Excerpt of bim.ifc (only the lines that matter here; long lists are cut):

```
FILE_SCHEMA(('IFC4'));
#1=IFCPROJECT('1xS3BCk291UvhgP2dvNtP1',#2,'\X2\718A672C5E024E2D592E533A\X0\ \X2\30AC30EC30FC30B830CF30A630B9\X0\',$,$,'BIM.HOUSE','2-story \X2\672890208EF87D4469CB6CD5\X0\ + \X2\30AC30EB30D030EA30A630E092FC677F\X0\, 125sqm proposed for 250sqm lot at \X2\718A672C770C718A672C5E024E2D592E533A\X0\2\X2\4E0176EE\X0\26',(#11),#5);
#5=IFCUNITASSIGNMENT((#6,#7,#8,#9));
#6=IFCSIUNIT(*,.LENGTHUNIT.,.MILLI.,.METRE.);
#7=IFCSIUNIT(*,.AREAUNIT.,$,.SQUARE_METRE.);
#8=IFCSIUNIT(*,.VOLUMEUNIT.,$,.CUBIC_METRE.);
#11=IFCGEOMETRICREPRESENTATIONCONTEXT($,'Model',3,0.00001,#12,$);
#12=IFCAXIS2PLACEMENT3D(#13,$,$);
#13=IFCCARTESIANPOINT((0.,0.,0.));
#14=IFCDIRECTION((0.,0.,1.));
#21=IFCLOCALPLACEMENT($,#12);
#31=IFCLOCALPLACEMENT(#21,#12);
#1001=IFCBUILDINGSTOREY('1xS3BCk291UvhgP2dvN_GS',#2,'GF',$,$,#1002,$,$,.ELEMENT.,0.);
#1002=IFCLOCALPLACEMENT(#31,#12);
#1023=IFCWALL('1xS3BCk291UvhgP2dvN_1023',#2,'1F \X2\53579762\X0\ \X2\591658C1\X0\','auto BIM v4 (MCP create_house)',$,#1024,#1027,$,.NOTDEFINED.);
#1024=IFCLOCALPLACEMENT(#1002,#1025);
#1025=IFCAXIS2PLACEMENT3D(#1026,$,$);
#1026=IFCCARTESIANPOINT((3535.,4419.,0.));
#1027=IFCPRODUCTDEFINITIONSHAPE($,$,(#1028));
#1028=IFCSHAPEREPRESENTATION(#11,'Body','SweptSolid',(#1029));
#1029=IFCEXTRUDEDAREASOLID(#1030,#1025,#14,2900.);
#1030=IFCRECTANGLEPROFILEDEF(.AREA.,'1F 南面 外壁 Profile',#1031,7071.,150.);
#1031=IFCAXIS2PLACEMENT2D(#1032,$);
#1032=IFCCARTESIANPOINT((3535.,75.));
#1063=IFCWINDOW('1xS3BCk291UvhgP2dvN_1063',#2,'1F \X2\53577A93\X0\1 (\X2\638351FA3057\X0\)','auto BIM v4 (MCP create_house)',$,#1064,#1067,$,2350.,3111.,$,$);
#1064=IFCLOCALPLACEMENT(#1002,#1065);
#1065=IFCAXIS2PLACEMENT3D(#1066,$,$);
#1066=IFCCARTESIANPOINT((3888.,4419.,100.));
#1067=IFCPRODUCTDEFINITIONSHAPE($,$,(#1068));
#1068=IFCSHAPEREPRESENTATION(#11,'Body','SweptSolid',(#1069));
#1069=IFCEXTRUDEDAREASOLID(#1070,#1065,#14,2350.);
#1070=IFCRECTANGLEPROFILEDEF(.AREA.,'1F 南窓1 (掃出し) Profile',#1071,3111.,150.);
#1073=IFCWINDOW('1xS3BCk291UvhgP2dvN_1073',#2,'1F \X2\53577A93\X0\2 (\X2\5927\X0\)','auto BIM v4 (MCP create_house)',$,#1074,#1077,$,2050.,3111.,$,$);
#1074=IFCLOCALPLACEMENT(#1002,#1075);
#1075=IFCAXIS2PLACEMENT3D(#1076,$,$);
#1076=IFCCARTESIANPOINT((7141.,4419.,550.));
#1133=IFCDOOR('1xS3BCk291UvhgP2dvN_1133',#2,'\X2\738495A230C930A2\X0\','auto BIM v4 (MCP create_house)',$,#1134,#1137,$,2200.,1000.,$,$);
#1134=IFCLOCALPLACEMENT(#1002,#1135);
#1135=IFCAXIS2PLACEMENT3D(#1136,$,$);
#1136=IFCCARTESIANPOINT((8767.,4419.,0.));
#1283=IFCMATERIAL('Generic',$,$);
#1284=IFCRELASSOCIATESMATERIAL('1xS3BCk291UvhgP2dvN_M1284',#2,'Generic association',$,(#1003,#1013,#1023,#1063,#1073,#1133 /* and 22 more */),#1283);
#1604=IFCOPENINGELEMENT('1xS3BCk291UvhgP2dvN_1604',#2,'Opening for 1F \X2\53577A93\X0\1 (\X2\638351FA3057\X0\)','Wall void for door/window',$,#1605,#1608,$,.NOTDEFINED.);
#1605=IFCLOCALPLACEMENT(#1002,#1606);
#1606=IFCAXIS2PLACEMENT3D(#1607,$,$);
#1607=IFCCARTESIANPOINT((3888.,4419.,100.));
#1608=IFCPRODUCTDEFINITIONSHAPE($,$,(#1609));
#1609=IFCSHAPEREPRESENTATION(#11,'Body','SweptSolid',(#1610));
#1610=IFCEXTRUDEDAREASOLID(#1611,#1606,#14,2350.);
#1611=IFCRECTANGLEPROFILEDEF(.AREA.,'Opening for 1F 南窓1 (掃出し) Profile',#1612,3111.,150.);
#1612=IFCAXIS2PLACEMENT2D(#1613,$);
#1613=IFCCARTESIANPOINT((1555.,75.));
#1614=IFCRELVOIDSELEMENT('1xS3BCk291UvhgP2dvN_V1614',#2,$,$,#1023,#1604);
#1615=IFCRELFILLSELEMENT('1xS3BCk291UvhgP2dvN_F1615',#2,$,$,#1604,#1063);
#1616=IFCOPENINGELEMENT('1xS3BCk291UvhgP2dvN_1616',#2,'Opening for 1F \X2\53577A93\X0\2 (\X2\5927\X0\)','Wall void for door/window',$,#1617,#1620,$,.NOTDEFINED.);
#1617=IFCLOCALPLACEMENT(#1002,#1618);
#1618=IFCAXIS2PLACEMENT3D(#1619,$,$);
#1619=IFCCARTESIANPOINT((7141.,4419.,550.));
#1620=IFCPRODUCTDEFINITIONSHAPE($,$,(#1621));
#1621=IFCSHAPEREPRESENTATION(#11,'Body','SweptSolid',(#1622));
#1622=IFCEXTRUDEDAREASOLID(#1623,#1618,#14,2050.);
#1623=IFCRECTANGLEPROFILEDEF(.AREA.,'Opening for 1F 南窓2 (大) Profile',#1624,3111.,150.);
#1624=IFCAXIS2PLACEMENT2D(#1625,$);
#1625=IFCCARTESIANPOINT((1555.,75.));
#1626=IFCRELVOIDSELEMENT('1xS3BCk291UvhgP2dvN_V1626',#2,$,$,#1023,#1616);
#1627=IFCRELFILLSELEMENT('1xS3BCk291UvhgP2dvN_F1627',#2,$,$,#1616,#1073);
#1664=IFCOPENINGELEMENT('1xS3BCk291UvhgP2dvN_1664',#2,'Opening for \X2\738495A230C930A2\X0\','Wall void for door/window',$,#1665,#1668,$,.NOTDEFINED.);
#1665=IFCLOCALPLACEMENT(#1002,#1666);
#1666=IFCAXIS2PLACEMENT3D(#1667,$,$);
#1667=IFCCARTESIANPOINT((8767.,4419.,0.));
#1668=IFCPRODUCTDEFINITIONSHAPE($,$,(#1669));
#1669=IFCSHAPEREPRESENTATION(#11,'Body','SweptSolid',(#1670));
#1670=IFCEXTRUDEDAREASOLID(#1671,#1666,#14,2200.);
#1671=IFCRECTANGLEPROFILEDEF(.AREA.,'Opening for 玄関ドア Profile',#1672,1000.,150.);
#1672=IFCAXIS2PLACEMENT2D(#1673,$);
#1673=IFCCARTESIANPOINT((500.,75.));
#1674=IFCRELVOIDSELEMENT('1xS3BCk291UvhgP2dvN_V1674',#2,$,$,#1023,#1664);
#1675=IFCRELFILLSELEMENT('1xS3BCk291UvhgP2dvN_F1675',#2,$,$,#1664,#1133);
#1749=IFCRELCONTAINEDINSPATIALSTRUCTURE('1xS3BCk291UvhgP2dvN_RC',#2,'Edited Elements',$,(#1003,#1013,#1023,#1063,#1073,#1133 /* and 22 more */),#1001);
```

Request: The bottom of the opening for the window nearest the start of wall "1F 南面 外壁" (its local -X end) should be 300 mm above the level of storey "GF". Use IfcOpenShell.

```python
import numpy as np
import ifcopenshell
import ifcopenshell.api.geometry
import ifcopenshell.geom
import ifcopenshell.util.element
import ifcopenshell.util.placement
import ifcopenshell.util.shape
import ifcopenshell.util.unit

model = ifcopenshell.open("bim.ifc")
unit_scale = ifcopenshell.util.unit.calculate_unit_scale(model)

window = model.by_guid("1xS3BCk291UvhgP2dvN_1063")
opening = window.FillsVoids[0].RelatingOpeningElement
storey = ifcopenshell.util.element.get_container(window, ifc_class="IfcBuildingStorey")
level = ifcopenshell.util.placement.get_local_placement(storey.ObjectPlacement)[2, 3]

# The opening's origin need not be at the sill, so measure its lowest point.
shape = ifcopenshell.geom.create_shape(ifcopenshell.geom.settings(), opening)
bottom = ifcopenshell.util.shape.get_shape_bottom_elevation(shape, shape.geometry) / unit_scale
dz = level + 0.3 / unit_scale - bottom

shift = np.array([0.0, 0.0, dz])
# The window is not placed relative to its opening, so move both.
for product in (opening, window):
    matrix = ifcopenshell.util.placement.get_local_placement(product.ObjectPlacement)
    matrix[:3, 3] += shift
    ifcopenshell.api.geometry.edit_object_placement(model, product=product, matrix=matrix, is_si=False)

print(f"moved by {dz * unit_scale:+.3f} m")

model.write("bim_v2.ifc")
```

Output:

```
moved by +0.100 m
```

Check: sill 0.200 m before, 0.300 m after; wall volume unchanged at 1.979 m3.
